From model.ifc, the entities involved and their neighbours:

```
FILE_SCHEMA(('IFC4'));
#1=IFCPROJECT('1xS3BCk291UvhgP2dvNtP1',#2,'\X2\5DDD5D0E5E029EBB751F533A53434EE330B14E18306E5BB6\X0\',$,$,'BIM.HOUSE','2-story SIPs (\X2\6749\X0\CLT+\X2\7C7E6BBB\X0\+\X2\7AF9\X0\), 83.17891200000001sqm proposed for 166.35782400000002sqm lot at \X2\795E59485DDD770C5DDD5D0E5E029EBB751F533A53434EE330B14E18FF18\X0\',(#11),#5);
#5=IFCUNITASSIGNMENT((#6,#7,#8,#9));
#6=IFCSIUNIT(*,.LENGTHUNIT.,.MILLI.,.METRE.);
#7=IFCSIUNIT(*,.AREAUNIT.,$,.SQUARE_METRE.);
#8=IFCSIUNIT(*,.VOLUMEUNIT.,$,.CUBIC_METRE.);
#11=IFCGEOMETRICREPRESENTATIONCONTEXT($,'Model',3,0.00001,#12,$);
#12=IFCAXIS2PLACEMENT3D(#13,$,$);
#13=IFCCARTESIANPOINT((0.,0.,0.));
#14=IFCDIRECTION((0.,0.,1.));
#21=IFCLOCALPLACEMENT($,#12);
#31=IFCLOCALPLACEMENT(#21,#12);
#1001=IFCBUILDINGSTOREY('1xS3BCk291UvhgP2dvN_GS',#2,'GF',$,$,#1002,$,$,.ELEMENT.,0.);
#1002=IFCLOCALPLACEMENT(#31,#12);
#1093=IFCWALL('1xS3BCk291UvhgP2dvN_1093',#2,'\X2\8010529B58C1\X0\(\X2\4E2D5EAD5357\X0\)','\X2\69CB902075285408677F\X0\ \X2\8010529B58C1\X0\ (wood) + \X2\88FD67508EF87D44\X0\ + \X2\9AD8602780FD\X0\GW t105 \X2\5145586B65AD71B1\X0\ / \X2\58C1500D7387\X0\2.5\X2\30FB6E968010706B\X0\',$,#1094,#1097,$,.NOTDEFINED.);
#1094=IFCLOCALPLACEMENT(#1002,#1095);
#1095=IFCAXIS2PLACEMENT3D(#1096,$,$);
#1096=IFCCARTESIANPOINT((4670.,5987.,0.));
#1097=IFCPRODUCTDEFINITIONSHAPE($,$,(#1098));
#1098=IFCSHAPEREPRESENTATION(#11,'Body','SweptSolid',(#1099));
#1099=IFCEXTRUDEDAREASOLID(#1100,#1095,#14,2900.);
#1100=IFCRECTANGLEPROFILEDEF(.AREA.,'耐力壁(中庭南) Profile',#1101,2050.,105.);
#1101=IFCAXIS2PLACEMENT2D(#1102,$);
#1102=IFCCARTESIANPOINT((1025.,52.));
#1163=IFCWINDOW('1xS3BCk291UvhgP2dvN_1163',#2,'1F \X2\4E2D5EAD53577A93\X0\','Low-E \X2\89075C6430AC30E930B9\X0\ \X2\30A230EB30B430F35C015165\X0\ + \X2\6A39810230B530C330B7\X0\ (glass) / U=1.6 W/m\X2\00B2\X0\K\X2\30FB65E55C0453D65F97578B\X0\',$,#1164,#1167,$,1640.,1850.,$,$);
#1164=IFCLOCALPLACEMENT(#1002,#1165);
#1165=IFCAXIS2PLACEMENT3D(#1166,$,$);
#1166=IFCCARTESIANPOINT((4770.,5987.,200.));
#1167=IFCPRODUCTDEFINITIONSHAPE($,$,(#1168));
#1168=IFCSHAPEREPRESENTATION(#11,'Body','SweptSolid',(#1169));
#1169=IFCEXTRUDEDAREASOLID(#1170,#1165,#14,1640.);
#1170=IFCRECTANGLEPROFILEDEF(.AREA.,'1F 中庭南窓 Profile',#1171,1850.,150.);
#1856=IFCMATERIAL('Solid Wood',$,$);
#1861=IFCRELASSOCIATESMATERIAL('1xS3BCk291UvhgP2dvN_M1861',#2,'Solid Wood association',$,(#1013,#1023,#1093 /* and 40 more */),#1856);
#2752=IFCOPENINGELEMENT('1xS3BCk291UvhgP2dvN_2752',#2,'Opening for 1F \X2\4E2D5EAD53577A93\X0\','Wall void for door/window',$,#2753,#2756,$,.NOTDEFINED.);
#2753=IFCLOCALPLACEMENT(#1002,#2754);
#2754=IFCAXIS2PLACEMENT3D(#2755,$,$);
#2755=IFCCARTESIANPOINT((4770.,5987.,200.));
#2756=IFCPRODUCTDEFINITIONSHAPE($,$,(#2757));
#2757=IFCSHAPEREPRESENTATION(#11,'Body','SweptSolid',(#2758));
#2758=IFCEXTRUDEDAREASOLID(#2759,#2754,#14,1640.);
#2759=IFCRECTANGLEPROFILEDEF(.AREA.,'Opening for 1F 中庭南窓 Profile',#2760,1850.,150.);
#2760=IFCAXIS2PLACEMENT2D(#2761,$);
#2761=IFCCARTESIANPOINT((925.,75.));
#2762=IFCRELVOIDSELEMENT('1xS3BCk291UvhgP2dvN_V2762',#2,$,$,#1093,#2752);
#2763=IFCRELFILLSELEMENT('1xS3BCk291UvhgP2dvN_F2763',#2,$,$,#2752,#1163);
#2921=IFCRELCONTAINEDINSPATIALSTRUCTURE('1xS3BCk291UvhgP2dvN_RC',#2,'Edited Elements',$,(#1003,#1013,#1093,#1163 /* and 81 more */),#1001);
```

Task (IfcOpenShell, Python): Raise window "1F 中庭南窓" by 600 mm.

```python
import numpy as np
import ifcopenshell
import ifcopenshell.api.geometry
import ifcopenshell.util.placement
import ifcopenshell.util.unit

model = ifcopenshell.open("model.ifc")
unit_scale = ifcopenshell.util.unit.calculate_unit_scale(model)

window = model.by_guid("1xS3BCk291UvhgP2dvN_1163")
opening = window.FillsVoids[0].RelatingOpeningElement
dz = 600.0

shift = np.array([0.0, 0.0, dz])
# The window is not placed relative to its opening, so move both.
for product in (opening, window):
    matrix = ifcopenshell.util.placement.get_local_placement(product.ObjectPlacement)
    matrix[:3, 3] += shift
    ifcopenshell.api.geometry.edit_object_placement(model, product=product, matrix=matrix, is_si=False)

print(f"moved by {dz * unit_scale:+.3f} m")

model.write("model_rev.ifc")
```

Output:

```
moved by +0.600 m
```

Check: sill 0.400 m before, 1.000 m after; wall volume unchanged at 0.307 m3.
